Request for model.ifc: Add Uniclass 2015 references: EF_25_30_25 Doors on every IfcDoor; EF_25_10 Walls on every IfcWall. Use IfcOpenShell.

First a look at what the model holds.

```python
import ifcopenshell

model = ifcopenshell.open("model.ifc")
print(model.schema)
print("classifications:", [c.Name for c in model.by_type("IfcClassification")])
for ifc_class in ("IfcDoor", "IfcRoof", "IfcStair", "IfcWall", "IfcWindow"):
    print(ifc_class, len(model.by_type(ifc_class)))
```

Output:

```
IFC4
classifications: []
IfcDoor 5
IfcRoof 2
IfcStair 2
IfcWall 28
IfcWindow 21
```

```python
import ifcopenshell
import ifcopenshell.api.classification

model = ifcopenshell.open("model.ifc")

system = ifcopenshell.api.classification.add_classification(model, classification="Uniclass 2015")

codes = {
    "IfcDoor": ("EF_25_30_25", "Doors"),
    "IfcWall": ("EF_25_10", "Walls"),
}
for ifc_class, (code, name) in codes.items():
    products = model.by_type(ifc_class)
    ifcopenshell.api.classification.add_reference(
        model, products=products, classification=system, identification=code, name=name
    )
    print(code, len(products))

model.write("model_updated.ifc")
```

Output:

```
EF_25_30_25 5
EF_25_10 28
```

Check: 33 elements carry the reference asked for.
